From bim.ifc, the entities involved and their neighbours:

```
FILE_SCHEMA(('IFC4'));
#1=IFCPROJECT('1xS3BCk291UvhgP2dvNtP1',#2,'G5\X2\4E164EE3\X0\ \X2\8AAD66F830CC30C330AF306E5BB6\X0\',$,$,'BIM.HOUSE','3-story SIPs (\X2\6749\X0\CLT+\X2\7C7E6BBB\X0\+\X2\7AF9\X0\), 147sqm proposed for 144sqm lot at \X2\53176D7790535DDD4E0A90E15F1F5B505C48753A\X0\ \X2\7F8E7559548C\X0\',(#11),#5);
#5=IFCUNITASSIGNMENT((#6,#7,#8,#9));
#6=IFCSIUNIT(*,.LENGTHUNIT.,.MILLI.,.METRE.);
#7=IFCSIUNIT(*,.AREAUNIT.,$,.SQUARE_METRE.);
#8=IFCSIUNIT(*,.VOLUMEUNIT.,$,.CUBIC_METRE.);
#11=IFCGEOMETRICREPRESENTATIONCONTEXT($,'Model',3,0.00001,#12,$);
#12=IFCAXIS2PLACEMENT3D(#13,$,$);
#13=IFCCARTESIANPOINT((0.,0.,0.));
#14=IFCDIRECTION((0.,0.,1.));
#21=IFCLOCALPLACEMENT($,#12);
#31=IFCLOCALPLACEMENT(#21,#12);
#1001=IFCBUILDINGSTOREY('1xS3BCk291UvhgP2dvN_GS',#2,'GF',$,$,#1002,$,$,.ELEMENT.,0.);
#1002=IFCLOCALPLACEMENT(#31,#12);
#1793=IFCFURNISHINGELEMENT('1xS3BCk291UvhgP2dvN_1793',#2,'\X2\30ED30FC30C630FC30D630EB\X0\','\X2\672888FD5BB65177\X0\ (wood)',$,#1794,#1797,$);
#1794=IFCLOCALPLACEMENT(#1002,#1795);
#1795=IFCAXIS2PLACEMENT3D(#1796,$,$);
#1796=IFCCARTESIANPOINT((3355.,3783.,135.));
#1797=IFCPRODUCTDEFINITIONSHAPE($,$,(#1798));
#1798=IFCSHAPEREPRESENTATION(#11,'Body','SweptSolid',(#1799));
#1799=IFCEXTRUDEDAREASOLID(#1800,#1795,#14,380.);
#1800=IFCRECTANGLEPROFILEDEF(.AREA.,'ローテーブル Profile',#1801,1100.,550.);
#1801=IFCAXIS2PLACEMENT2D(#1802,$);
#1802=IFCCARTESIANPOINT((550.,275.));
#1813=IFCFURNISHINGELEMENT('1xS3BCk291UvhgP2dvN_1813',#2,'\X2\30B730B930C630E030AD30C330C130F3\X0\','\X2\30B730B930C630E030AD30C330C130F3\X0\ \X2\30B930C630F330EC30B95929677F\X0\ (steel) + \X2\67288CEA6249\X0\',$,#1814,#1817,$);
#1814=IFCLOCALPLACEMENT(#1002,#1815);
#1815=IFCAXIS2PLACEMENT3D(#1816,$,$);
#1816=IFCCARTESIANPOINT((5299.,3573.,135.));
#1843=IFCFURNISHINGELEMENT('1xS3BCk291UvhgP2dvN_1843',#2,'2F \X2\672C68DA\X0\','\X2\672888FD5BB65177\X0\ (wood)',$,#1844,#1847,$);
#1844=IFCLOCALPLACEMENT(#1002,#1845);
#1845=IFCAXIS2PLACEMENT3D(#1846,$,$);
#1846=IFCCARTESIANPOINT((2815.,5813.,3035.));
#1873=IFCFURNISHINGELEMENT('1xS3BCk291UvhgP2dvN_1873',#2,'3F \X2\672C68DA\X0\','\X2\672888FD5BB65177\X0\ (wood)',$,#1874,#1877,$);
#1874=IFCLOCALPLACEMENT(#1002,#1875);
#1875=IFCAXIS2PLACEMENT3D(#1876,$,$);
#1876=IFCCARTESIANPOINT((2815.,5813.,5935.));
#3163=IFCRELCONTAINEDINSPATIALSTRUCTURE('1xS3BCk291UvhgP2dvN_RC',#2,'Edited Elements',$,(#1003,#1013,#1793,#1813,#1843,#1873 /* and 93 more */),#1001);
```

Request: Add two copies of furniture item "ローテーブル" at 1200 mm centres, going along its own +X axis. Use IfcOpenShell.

```python
import ifcopenshell
import ifcopenshell.api.geometry
import ifcopenshell.api.root
import ifcopenshell.util.element
import ifcopenshell.util.placement
import ifcopenshell.util.unit

model = ifcopenshell.open("bim.ifc")
unit_scale = ifcopenshell.util.unit.calculate_unit_scale(model)


def reuse_history(source, copy):
    """copy_class also copies each property set's owner history, people and application; keep the originals."""
    for rel in copy.IsDefinedBy:
        if rel.is_a("IfcRelDefinesByProperties") and (history := rel.RelatingPropertyDefinition.OwnerHistory):
            rel.RelatingPropertyDefinition.OwnerHistory = source.OwnerHistory
            ifcopenshell.util.element.remove_deep2(model, history)


source = model.by_guid("1xS3BCk291UvhgP2dvN_1793")
base = ifcopenshell.util.placement.get_local_placement(source.ObjectPlacement)
step = base[:3, 0] * 1.2 / unit_scale

for i in range(1, 3):
    copy = ifcopenshell.api.root.copy_class(model, product=source)
    copy.Representation = ifcopenshell.util.element.copy_deep(
        model, source.Representation, exclude=["IfcGeometricRepresentationContext", "IfcRepresentationMap"]
    )
    reuse_history(source, copy)
    matrix = base.copy()
    matrix[:3, 3] += i * step
    print("added at", matrix[:3, 3].round(3) + 0.0)
    ifcopenshell.api.geometry.edit_object_placement(model, product=copy, matrix=matrix, is_si=False)

model.write("bim_rev.ifc")
```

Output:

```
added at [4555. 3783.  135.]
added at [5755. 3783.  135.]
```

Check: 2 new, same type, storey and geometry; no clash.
